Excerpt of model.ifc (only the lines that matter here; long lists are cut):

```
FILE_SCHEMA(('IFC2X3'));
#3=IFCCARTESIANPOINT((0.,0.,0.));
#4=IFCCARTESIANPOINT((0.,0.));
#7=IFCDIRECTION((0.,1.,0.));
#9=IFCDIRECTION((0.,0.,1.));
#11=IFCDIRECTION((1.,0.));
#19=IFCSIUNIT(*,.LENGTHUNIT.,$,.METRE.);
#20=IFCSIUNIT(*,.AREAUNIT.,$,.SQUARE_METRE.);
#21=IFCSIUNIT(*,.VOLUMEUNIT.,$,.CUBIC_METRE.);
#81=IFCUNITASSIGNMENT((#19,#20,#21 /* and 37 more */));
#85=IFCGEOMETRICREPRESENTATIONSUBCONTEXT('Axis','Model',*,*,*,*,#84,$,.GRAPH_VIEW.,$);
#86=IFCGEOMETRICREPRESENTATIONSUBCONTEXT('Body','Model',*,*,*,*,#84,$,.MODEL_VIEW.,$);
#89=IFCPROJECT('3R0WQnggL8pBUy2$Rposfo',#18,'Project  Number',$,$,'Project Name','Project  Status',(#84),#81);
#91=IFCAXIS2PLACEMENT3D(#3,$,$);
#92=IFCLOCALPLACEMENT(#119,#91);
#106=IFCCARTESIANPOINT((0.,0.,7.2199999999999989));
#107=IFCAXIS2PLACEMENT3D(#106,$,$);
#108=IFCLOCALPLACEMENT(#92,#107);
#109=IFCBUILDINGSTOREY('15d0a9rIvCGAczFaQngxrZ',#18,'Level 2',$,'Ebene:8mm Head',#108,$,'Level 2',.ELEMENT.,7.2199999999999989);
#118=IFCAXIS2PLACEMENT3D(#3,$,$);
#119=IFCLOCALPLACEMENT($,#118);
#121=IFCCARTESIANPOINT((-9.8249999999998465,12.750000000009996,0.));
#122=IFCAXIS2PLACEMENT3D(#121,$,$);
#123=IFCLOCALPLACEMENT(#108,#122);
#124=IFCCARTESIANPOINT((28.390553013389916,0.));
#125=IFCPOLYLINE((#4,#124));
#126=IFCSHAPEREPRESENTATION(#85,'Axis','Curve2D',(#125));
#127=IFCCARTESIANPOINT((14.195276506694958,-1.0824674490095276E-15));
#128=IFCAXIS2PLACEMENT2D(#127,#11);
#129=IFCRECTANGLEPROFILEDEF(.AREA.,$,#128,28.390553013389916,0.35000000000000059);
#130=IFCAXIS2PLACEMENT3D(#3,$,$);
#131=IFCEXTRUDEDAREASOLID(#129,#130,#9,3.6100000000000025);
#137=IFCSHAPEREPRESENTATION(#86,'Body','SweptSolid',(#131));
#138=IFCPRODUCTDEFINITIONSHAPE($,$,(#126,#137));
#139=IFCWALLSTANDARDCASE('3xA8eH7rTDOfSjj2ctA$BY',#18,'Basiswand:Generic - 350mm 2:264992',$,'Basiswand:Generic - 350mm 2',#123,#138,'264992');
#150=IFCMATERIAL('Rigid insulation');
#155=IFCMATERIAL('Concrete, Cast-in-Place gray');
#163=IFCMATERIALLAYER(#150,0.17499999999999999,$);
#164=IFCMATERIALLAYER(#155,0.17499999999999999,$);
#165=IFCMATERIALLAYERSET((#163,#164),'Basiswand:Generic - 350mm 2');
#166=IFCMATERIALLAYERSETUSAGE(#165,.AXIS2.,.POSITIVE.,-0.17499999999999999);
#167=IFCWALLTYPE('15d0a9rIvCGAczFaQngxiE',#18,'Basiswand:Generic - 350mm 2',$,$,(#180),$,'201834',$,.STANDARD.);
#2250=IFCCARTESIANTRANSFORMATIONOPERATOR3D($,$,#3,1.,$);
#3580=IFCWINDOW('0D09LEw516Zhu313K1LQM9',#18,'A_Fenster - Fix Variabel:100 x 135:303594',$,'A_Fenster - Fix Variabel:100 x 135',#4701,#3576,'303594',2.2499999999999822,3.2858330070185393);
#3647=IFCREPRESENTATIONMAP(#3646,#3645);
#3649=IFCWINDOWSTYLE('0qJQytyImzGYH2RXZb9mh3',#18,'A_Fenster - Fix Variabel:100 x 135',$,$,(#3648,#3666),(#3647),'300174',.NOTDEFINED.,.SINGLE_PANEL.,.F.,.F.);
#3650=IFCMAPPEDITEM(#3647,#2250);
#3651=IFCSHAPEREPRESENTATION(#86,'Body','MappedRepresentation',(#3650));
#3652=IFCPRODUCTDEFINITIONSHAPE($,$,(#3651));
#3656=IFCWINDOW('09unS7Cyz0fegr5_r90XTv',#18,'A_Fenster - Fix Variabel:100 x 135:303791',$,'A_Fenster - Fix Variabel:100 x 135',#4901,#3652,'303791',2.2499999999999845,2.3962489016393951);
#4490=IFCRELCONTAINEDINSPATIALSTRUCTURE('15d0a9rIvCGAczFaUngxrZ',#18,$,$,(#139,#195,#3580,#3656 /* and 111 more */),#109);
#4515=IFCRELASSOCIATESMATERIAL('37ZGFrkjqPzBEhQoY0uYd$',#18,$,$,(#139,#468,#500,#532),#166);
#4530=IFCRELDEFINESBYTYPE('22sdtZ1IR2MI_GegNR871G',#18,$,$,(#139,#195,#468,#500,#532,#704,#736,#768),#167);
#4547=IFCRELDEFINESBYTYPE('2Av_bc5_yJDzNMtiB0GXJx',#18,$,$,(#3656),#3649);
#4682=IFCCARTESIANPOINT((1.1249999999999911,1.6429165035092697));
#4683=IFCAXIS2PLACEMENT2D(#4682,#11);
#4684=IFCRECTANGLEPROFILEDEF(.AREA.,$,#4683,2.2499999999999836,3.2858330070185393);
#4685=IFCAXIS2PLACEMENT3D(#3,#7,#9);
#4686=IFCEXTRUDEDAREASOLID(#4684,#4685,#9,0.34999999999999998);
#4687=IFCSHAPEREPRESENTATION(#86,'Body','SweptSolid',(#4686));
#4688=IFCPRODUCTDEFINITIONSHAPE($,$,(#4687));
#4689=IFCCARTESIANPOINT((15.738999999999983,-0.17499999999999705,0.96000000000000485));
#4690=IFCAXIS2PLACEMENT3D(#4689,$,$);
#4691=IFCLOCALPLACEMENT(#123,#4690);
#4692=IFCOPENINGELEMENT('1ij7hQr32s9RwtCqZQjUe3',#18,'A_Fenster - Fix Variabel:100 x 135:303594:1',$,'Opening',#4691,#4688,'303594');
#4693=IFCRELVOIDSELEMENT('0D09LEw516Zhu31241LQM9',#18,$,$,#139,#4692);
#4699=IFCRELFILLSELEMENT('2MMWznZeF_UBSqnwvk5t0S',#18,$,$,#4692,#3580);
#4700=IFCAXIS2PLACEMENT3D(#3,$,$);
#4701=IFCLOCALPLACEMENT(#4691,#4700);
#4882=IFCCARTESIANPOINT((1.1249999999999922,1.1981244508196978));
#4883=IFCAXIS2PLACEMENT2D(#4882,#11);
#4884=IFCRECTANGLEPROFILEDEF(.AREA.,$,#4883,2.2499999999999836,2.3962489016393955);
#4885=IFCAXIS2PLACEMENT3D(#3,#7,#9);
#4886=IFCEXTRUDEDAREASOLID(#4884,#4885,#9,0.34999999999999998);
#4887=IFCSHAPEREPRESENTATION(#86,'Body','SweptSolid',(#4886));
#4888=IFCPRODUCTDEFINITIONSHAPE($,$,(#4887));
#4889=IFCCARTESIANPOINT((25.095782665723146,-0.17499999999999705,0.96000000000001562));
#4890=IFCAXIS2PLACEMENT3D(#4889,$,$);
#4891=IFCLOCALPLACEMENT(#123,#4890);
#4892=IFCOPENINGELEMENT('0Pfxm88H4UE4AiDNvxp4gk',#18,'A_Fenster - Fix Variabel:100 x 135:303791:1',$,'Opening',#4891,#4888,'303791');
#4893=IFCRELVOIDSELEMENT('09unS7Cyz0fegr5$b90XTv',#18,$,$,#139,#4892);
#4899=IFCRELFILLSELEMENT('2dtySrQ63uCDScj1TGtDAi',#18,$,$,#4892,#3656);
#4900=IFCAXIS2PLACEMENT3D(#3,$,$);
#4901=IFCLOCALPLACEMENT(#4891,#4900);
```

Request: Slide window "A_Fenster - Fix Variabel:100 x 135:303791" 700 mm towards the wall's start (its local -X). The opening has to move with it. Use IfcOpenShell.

```python
import ifcopenshell
import ifcopenshell.api.geometry
import ifcopenshell.util.placement

model = ifcopenshell.open("model.ifc")

window = model.by_id(3656)
opening = window.FillsVoids[0].RelatingOpeningElement
wall = opening.VoidsElements[0].RelatingBuildingElement

wall_matrix = ifcopenshell.util.placement.get_local_placement(wall.ObjectPlacement)
shift = wall_matrix[:3, 0] * -0.7
before = ifcopenshell.util.placement.get_local_placement(window.ObjectPlacement)[:3, 3].copy()

# The window is placed relative to its opening, so it follows when the opening moves.
matrix = ifcopenshell.util.placement.get_local_placement(opening.ObjectPlacement)
matrix[:3, 3] += shift
ifcopenshell.api.geometry.edit_object_placement(
    model, product=opening, matrix=matrix, is_si=False, should_transform_children=True
)

after = ifcopenshell.util.placement.get_local_placement(window.ObjectPlacement)[:3, 3]
print("window moved by", (after - before).round(3) + 0.0)

model.write("model_updated.ifc")
```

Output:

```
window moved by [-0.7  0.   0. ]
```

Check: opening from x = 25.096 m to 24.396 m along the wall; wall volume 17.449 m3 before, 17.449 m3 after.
